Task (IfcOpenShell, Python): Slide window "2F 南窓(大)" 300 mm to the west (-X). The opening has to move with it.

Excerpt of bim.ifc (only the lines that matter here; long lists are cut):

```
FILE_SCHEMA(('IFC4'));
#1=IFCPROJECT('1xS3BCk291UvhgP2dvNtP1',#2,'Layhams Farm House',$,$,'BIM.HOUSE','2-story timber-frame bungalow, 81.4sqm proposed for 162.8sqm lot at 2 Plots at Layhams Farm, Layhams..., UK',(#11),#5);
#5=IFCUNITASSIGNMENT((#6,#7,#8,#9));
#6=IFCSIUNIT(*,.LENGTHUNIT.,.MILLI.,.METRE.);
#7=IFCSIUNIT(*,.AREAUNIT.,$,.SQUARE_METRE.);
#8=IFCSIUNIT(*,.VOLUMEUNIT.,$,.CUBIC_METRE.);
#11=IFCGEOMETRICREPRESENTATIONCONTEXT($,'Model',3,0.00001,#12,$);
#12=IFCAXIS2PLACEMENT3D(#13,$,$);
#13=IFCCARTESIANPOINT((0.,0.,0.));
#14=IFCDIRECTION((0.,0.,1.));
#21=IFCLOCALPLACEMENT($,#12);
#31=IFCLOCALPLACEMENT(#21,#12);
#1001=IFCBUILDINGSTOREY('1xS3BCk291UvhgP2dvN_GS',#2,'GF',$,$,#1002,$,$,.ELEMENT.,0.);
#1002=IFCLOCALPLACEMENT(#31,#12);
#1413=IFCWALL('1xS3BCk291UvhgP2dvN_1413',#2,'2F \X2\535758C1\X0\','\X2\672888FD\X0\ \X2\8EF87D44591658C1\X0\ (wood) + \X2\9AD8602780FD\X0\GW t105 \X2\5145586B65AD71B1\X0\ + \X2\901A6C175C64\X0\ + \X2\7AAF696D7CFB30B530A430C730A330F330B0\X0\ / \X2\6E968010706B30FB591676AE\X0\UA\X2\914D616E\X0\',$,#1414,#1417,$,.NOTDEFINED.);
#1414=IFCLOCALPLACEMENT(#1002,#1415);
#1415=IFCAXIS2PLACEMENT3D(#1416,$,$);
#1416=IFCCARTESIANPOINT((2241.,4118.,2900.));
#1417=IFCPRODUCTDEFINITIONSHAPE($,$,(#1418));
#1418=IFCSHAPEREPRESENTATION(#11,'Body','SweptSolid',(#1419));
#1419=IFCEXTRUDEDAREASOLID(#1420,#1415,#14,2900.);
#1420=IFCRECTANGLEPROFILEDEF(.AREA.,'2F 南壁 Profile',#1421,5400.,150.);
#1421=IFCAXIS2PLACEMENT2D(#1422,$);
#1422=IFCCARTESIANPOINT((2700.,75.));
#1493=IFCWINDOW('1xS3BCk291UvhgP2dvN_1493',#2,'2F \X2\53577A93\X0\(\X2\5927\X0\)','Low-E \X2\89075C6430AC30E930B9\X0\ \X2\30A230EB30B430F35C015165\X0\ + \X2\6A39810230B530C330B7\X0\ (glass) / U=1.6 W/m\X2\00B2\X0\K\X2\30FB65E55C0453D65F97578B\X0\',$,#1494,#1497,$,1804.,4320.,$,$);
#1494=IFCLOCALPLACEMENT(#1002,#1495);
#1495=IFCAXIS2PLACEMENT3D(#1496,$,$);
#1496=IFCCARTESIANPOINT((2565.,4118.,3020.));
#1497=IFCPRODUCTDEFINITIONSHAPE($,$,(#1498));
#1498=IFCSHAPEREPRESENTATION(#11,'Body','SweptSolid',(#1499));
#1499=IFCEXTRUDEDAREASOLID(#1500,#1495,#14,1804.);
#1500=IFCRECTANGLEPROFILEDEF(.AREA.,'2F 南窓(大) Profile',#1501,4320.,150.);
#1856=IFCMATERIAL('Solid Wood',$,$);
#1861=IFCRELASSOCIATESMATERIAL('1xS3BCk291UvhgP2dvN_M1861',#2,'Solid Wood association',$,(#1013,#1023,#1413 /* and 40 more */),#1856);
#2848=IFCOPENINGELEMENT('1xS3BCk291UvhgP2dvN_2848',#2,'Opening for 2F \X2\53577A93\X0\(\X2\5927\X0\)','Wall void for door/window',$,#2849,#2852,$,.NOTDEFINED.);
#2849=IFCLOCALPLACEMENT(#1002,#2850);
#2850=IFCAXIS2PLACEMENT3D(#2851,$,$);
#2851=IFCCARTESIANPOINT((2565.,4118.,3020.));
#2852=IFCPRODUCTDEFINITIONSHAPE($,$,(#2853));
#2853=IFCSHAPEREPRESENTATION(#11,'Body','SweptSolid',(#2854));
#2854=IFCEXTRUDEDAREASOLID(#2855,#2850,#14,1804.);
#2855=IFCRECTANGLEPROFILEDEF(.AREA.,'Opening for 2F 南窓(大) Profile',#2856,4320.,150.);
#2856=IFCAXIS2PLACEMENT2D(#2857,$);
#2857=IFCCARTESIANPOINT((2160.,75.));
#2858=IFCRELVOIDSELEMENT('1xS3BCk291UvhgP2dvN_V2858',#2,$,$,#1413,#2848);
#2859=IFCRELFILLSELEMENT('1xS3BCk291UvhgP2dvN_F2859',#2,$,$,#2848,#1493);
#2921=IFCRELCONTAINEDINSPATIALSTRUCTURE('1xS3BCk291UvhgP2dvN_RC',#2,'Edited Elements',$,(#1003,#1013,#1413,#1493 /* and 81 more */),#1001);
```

```python
import ifcopenshell
import ifcopenshell.api.geometry
import ifcopenshell.util.placement
import ifcopenshell.util.unit

model = ifcopenshell.open("bim.ifc")
unit_scale = ifcopenshell.util.unit.calculate_unit_scale(model)

window = model.by_id(1493)
opening = window.FillsVoids[0].RelatingOpeningElement
wall = opening.VoidsElements[0].RelatingBuildingElement

wall_matrix = ifcopenshell.util.placement.get_local_placement(wall.ObjectPlacement)
shift = wall_matrix[:3, 0] * -0.3 / unit_scale
before = ifcopenshell.util.placement.get_local_placement(window.ObjectPlacement)[:3, 3].copy()

# The window is not placed relative to its opening, so move both.
for product in (opening, window):
    matrix = ifcopenshell.util.placement.get_local_placement(product.ObjectPlacement)
    matrix[:3, 3] += shift
    ifcopenshell.api.geometry.edit_object_placement(model, product=product, matrix=matrix, is_si=False)

after = ifcopenshell.util.placement.get_local_placement(window.ObjectPlacement)[:3, 3]
print("window moved by", (after - before).round(3) + 0.0)

model.write("bim_updated.ifc")
```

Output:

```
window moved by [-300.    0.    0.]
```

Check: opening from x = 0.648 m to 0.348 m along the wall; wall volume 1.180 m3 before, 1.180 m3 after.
